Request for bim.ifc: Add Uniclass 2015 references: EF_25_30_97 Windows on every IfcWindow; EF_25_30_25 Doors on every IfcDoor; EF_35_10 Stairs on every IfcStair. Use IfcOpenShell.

First a look at what the model holds.

```python
import ifcopenshell

model = ifcopenshell.open("bim.ifc")
print(model.schema)
print("classifications:", [c.Name for c in model.by_type("IfcClassification")])
for ifc_class in ("IfcDoor", "IfcRoof", "IfcStair", "IfcWall", "IfcWindow"):
    print(ifc_class, len(model.by_type(ifc_class)))
```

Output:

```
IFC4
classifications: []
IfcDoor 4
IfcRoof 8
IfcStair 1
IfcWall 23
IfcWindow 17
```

```python
import ifcopenshell
import ifcopenshell.api.classification

model = ifcopenshell.open("bim.ifc")

system = ifcopenshell.api.classification.add_classification(model, classification="Uniclass 2015")

codes = {
    "IfcWindow": ("EF_25_30_97", "Windows"),
    "IfcDoor": ("EF_25_30_25", "Doors"),
    "IfcStair": ("EF_35_10", "Stairs"),
}
for ifc_class, (code, name) in codes.items():
    products = model.by_type(ifc_class)
    ifcopenshell.api.classification.add_reference(
        model, products=products, classification=system, identification=code, name=name
    )
    print(code, len(products))

model.write("bim_updated.ifc")
```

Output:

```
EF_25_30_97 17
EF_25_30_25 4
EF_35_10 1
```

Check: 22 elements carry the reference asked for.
